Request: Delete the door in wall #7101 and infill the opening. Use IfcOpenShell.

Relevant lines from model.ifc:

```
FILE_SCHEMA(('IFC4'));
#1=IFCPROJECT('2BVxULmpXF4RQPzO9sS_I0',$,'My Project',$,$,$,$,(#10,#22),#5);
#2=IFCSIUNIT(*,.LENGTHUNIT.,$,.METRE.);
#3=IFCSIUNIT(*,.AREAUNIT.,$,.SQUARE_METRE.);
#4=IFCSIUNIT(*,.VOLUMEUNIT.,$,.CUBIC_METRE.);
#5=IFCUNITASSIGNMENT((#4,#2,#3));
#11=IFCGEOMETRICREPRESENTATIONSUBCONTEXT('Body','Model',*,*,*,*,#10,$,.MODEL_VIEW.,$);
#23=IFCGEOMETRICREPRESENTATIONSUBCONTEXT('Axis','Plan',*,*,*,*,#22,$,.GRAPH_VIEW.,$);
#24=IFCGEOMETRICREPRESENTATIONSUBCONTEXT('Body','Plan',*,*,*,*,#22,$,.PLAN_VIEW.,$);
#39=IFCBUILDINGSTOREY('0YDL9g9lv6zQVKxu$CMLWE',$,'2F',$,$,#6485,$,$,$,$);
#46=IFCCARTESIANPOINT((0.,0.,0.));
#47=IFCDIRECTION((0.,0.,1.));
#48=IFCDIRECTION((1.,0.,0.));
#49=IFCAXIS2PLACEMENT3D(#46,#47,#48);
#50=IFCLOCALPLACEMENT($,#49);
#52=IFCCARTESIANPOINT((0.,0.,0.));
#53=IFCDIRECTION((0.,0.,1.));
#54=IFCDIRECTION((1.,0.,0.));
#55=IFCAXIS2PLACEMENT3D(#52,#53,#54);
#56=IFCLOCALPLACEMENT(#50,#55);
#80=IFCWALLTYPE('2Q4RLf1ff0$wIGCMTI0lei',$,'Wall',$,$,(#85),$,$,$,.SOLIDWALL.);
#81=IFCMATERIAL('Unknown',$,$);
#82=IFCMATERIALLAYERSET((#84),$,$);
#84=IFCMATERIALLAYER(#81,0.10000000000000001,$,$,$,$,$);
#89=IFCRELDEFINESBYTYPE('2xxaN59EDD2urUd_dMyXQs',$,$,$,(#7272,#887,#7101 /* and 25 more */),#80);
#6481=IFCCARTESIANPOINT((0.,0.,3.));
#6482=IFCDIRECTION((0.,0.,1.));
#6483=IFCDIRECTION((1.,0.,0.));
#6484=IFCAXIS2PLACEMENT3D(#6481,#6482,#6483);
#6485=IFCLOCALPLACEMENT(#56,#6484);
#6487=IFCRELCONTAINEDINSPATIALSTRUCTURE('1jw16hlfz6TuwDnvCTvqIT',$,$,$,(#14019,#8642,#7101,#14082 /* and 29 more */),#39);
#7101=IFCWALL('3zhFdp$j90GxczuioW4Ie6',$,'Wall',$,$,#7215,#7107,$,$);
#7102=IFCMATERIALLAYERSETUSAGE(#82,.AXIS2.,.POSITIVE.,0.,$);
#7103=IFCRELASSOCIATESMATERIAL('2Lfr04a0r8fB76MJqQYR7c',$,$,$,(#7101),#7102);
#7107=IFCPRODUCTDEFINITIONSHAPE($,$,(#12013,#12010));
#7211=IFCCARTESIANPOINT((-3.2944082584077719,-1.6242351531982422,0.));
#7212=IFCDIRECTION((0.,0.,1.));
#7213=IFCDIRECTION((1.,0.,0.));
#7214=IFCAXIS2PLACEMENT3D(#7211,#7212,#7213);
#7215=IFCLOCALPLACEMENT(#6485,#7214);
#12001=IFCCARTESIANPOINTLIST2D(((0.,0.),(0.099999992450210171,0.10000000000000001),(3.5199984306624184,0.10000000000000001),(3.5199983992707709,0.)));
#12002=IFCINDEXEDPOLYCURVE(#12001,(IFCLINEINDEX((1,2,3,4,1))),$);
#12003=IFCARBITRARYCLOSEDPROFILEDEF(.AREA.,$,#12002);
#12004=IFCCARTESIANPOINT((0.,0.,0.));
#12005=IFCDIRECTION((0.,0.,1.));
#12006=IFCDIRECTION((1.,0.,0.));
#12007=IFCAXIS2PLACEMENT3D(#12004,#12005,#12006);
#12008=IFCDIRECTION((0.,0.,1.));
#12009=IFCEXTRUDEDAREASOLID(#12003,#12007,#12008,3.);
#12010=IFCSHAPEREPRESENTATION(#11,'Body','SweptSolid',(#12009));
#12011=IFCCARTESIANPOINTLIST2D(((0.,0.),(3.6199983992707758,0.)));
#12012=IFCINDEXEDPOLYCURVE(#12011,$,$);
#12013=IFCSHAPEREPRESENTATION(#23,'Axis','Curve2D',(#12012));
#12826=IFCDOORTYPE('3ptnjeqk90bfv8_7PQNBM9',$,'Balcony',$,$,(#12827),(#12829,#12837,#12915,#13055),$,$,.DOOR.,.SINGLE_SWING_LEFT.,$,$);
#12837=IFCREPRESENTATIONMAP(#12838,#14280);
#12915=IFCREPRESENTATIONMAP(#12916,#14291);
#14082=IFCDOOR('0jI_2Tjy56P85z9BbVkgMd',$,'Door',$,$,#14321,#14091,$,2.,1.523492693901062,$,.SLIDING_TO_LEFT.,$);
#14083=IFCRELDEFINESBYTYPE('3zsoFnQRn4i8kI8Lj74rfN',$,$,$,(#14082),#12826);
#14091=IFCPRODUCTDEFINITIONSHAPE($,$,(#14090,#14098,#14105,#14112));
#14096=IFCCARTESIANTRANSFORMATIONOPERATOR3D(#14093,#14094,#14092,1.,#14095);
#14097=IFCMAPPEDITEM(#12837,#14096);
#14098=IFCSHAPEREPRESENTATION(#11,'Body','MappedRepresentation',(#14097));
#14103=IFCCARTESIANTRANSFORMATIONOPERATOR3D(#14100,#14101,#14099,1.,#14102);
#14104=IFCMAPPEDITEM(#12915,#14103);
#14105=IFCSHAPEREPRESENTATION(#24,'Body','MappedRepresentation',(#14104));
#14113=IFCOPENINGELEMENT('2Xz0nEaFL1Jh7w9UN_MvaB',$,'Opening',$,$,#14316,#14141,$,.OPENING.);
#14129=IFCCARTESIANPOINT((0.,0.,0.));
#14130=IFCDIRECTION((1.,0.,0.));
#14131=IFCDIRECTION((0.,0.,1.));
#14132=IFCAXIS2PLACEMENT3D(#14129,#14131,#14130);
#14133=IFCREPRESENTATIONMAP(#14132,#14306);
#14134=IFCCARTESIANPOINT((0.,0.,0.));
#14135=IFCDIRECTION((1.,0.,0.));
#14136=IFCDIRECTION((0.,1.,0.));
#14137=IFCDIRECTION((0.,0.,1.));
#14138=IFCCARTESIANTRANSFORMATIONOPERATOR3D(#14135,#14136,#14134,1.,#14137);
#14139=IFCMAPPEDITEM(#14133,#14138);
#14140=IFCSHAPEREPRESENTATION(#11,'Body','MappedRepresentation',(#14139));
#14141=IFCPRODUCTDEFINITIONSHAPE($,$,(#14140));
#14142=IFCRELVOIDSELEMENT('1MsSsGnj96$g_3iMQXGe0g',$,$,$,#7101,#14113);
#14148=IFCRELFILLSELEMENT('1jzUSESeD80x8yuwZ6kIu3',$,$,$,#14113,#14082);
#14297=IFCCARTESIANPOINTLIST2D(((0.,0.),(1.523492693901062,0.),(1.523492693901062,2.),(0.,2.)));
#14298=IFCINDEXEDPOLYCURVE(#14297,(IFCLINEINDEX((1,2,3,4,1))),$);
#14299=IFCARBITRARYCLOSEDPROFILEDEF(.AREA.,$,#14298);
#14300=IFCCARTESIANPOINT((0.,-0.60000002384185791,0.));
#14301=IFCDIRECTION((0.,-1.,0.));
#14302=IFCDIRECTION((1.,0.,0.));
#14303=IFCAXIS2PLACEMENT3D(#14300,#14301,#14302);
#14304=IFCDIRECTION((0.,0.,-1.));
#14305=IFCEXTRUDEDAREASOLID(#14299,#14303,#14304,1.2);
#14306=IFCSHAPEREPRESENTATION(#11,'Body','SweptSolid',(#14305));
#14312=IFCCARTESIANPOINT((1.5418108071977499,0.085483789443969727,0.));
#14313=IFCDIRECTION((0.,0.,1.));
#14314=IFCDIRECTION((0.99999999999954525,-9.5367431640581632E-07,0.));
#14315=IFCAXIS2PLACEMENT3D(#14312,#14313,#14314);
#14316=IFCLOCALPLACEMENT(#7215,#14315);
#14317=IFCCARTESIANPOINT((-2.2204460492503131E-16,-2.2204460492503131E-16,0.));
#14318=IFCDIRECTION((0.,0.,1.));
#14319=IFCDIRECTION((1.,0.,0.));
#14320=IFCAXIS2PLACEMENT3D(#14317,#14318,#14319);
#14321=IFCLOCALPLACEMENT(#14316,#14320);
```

```python
import ifcopenshell
import ifcopenshell.api.feature
import ifcopenshell.api.root
import ifcopenshell.geom
import ifcopenshell.util.shape

model = ifcopenshell.open("model.ifc")
settings = ifcopenshell.geom.settings()


def volume(element):
    """Net volume in cubic metres, openings subtracted."""
    shape = ifcopenshell.geom.create_shape(settings, element)
    return ifcopenshell.util.shape.get_volume(shape.geometry)


door = model.by_guid("0jI_2Tjy56P85z9BbVkgMd")
opening = door.FillsVoids[0].RelatingOpeningElement
wall = opening.VoidsElements[0].RelatingBuildingElement
before = volume(wall)

ifcopenshell.api.root.remove_product(model, product=door)
ifcopenshell.api.feature.remove_feature(model, feature=opening)

after = volume(wall)

print(f"wall volume {before:.3f} -> {after:.3f} m3")

model.write("model_rev.ifc")
```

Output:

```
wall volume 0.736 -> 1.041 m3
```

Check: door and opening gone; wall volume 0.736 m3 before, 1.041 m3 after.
